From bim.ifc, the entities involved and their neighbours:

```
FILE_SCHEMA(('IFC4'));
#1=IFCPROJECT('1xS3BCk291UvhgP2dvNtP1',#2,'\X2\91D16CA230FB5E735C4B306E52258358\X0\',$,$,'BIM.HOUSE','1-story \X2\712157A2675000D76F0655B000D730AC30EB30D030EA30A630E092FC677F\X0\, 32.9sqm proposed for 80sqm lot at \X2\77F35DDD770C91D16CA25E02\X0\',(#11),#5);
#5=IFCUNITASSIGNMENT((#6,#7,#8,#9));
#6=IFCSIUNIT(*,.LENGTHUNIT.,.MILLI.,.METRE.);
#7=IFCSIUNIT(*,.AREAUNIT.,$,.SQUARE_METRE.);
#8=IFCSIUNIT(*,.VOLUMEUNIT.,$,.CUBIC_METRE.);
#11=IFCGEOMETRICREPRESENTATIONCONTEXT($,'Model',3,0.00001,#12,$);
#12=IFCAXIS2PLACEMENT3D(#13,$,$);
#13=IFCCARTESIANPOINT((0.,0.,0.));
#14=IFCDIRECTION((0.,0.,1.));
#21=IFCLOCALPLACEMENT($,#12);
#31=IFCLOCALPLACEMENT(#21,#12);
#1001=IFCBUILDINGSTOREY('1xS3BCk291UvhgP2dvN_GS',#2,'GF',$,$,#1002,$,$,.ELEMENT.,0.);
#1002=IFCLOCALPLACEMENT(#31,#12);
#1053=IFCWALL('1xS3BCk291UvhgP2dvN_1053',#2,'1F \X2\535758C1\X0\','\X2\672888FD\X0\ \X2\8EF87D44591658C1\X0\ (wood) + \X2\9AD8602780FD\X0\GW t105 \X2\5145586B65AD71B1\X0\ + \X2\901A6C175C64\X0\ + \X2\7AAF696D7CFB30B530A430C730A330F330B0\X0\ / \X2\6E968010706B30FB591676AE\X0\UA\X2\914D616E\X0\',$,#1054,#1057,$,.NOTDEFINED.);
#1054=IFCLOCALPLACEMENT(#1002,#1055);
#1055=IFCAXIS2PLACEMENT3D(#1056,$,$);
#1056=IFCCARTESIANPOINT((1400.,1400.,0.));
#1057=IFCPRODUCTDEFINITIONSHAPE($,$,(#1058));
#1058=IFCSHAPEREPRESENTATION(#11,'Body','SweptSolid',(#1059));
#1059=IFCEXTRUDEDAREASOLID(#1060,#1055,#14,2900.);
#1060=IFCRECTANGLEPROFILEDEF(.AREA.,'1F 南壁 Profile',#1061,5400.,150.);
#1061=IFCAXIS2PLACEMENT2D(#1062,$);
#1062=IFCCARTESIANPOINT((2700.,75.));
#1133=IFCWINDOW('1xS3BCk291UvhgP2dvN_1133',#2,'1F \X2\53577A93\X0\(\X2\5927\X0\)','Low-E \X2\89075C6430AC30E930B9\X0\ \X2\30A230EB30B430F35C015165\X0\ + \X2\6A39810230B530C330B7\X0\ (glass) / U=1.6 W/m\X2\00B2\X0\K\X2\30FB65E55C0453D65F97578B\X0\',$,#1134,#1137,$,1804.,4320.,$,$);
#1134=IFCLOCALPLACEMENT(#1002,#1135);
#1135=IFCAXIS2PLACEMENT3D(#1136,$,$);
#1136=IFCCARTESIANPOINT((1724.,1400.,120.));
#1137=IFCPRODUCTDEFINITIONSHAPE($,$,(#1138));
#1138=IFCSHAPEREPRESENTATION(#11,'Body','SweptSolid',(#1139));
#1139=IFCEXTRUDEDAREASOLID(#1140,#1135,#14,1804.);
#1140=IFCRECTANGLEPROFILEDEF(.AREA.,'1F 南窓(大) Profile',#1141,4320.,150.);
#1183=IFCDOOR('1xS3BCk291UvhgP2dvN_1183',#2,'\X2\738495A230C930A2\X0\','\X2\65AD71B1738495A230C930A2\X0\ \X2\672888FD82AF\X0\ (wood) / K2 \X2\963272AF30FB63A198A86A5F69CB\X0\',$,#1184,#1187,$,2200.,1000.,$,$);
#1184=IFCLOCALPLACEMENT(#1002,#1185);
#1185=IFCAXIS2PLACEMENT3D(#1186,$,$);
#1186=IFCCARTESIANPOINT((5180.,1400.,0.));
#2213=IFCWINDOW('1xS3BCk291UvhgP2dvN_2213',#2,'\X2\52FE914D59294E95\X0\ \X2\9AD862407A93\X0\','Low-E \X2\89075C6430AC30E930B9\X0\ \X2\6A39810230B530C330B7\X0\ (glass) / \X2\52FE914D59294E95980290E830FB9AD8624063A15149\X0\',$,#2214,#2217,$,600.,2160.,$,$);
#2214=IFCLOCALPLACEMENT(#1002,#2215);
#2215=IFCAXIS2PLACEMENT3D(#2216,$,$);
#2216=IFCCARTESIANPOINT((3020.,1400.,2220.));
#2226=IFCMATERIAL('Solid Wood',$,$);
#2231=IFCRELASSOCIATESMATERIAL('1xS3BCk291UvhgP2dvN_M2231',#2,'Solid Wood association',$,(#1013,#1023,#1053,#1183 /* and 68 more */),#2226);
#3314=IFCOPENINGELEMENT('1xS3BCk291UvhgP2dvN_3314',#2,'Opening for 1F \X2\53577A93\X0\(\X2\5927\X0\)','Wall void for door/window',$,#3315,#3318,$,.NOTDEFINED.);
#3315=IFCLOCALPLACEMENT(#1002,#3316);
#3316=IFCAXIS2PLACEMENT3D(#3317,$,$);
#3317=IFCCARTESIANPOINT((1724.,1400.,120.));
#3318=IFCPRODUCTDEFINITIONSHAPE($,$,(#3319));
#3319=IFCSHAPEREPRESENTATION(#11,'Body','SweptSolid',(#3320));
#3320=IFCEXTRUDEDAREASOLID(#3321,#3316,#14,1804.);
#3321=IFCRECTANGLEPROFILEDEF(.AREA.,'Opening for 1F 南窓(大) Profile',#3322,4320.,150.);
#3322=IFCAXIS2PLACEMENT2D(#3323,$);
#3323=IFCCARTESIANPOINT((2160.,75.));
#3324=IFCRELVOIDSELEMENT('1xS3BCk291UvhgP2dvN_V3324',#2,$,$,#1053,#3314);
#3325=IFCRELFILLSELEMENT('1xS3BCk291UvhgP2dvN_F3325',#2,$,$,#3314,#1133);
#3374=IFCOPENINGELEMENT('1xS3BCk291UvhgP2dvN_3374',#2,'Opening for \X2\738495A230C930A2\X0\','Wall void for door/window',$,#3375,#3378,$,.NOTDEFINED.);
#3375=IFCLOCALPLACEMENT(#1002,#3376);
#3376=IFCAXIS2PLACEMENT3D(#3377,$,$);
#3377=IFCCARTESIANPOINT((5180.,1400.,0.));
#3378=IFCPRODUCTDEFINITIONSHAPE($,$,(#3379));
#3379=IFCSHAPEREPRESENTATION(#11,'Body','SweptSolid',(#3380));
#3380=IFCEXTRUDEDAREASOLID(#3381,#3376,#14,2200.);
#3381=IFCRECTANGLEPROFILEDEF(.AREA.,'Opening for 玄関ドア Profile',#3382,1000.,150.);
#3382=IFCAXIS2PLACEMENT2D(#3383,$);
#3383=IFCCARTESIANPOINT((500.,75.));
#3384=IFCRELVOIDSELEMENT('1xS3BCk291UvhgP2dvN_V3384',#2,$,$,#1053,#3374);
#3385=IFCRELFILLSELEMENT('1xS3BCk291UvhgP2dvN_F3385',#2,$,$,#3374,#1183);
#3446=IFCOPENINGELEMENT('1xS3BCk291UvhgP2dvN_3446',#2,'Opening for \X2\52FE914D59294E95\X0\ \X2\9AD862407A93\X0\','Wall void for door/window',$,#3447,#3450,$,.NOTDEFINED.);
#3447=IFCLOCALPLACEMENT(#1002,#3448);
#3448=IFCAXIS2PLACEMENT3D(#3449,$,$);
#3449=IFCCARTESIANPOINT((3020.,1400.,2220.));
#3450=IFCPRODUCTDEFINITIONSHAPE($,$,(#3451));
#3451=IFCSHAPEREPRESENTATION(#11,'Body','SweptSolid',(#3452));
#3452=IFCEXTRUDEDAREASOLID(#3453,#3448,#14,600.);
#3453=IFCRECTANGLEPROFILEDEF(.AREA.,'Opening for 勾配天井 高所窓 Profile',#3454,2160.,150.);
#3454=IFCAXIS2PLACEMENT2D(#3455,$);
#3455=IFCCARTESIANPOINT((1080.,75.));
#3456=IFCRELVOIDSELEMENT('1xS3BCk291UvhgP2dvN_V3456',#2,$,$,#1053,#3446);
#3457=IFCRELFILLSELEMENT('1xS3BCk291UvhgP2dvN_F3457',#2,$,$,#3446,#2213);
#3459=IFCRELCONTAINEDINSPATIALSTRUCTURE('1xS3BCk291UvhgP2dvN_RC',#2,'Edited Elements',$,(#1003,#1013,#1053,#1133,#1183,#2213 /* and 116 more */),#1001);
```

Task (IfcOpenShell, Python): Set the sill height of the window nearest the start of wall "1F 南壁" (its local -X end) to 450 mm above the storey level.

```python
import numpy as np
import ifcopenshell
import ifcopenshell.api.geometry
import ifcopenshell.geom
import ifcopenshell.util.element
import ifcopenshell.util.placement
import ifcopenshell.util.shape
import ifcopenshell.util.unit

model = ifcopenshell.open("bim.ifc")
unit_scale = ifcopenshell.util.unit.calculate_unit_scale(model)

window = model.by_guid("1xS3BCk291UvhgP2dvN_1133")
opening = window.FillsVoids[0].RelatingOpeningElement
storey = ifcopenshell.util.element.get_container(window, ifc_class="IfcBuildingStorey")
level = ifcopenshell.util.placement.get_local_placement(storey.ObjectPlacement)[2, 3]

# The opening's origin need not be at the sill, so measure its lowest point.
shape = ifcopenshell.geom.create_shape(ifcopenshell.geom.settings(), opening)
bottom = ifcopenshell.util.shape.get_shape_bottom_elevation(shape, shape.geometry) / unit_scale
dz = level + 0.45 / unit_scale - bottom

shift = np.array([0.0, 0.0, dz])
# The window is not placed relative to its opening, so move both.
for product in (opening, window):
    matrix = ifcopenshell.util.placement.get_local_placement(product.ObjectPlacement)
    matrix[:3, 3] += shift
    ifcopenshell.api.geometry.edit_object_placement(model, product=product, matrix=matrix, is_si=False)

print(f"moved by {dz * unit_scale:+.3f} m")

model.write("bim_updated.ifc")
```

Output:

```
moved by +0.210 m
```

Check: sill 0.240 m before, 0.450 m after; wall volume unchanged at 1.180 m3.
